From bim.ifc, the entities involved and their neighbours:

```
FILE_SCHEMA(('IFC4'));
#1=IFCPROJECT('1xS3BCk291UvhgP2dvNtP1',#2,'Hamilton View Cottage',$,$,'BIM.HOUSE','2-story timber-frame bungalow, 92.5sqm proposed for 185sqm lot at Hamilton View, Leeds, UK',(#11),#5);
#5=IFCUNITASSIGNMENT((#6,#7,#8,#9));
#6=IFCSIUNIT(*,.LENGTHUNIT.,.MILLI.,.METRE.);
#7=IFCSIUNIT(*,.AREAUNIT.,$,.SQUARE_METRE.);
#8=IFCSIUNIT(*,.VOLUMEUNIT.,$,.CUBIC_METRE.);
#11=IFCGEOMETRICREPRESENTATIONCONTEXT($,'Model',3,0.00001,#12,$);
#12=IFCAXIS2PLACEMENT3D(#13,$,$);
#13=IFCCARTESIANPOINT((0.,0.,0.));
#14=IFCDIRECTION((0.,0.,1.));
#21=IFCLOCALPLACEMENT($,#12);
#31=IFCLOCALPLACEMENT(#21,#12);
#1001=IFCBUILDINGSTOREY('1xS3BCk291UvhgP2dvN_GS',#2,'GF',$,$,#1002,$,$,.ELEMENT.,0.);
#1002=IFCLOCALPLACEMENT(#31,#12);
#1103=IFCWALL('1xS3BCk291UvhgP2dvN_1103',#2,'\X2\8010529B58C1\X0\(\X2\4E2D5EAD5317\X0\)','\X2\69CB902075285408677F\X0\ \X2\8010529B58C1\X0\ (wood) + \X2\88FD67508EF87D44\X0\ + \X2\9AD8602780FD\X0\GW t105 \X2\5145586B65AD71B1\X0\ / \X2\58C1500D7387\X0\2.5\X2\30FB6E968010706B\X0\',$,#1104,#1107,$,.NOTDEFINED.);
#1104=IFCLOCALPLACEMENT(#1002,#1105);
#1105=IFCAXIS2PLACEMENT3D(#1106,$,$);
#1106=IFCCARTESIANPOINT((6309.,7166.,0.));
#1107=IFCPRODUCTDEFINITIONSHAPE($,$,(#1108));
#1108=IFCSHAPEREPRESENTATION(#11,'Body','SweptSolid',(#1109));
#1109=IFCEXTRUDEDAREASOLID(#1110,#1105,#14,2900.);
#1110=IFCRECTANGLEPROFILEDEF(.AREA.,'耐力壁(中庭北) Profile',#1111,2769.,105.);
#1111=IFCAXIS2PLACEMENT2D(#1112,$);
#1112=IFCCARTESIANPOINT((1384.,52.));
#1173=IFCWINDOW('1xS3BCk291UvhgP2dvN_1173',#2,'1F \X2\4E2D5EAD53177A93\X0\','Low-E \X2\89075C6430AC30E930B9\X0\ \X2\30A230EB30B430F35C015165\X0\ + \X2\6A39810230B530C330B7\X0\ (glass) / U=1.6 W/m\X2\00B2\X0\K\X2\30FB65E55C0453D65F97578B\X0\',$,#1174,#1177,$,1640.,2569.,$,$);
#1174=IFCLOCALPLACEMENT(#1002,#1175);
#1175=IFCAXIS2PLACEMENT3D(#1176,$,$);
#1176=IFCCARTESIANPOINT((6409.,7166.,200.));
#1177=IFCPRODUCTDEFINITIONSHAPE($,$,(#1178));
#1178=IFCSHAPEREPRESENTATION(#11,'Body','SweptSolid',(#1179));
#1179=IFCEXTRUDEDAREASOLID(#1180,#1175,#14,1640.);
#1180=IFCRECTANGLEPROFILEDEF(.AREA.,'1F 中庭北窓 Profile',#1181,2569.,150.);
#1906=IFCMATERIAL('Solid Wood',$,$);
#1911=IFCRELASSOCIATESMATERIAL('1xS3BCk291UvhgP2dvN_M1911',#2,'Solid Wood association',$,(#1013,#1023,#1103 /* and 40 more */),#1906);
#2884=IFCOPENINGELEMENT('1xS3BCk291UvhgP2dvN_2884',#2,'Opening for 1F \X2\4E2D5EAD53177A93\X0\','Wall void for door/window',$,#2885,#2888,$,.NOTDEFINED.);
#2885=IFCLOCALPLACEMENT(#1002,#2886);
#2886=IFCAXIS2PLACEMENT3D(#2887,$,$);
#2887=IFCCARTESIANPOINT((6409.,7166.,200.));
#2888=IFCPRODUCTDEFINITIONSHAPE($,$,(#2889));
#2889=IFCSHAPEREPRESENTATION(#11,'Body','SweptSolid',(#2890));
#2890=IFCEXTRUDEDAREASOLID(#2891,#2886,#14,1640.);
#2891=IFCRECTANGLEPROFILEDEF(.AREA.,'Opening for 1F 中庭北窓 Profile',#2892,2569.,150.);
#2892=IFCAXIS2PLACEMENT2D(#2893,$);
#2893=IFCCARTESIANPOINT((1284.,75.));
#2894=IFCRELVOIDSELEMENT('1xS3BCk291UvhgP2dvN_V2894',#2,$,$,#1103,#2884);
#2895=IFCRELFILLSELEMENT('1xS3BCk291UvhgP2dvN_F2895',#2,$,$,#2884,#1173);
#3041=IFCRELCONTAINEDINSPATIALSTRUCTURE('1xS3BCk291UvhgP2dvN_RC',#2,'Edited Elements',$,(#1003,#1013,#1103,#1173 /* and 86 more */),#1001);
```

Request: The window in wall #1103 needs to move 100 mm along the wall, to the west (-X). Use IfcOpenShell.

```python
import ifcopenshell
import ifcopenshell.api.geometry
import ifcopenshell.util.placement
import ifcopenshell.util.unit

model = ifcopenshell.open("bim.ifc")
unit_scale = ifcopenshell.util.unit.calculate_unit_scale(model)

window = model.by_id(1173)
opening = window.FillsVoids[0].RelatingOpeningElement
wall = opening.VoidsElements[0].RelatingBuildingElement

wall_matrix = ifcopenshell.util.placement.get_local_placement(wall.ObjectPlacement)
shift = wall_matrix[:3, 0] * -0.1 / unit_scale
before = ifcopenshell.util.placement.get_local_placement(window.ObjectPlacement)[:3, 3].copy()

# The window is not placed relative to its opening, so move both.
for product in (opening, window):
    matrix = ifcopenshell.util.placement.get_local_placement(product.ObjectPlacement)
    matrix[:3, 3] += shift
    ifcopenshell.api.geometry.edit_object_placement(model, product=product, matrix=matrix, is_si=False)

after = ifcopenshell.util.placement.get_local_placement(window.ObjectPlacement)[:3, 3]
print("window moved by", (after - before).round(3) + 0.0)

model.write("bim_updated.ifc")
```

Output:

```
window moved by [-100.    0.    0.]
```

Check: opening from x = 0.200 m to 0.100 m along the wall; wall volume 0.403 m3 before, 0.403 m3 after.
